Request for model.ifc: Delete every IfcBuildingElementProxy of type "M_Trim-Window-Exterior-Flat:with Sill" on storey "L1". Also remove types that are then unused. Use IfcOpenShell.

First a look at what the model holds.

```python
import ifcopenshell
import ifcopenshell.util.element

model = ifcopenshell.open("model.ifc")
print(model.schema)
storey = next(s for s in model.by_type("IfcBuildingStorey") if s.Name == "L1")
proxies = [e for e in ifcopenshell.util.element.get_decomposition(storey) if e.is_a("IfcBuildingElementProxy")]
seen = {}
for e in proxies:
    element_type = ifcopenshell.util.element.get_type(e)
    name = element_type.Name if element_type not in (None, e) else None
    seen[name] = seen.get(name, 0) + 1
for name, count in sorted(seen.items(), key=str):
    print(count, "x", name)
```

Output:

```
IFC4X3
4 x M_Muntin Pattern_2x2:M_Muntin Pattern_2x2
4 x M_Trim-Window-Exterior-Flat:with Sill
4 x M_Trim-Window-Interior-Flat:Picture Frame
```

```python
import ifcopenshell
import ifcopenshell.api.root
import ifcopenshell.util.element

model = ifcopenshell.open("model.ifc")

storey = next(s for s in model.by_type("IfcBuildingStorey") if s.Name == "L1")
proxies = [e for e in ifcopenshell.util.element.get_decomposition(storey) if e.is_a("IfcBuildingElementProxy")]
targets = [e for e in proxies if (t := ifcopenshell.util.element.get_type(e)) not in (None, e) and t.Name == "M_Trim-Window-Exterior-Flat:with Sill"]
types = {ifcopenshell.util.element.get_type(e) for e in targets} - {None, *targets}

for e in targets:
    ifcopenshell.api.root.remove_product(model, product=e)
print(len(targets), "removed")

unused = [t for t in types if not ifcopenshell.util.element.get_types(t)]
for t in unused:
    ifcopenshell.api.root.remove_product(model, product=t)
print(len(unused), "unused types removed")

model.write("model_rev.ifc")
```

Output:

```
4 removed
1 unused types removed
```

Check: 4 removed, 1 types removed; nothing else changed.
